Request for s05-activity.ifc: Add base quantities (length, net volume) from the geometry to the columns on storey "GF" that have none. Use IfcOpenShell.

First a look at what the model holds.

```python
import ifcopenshell
import ifcopenshell.util.element
import ifcopenshell.util.unit

model = ifcopenshell.open("s05-activity.ifc")
print(model.schema)
for unit_type in ("LENGTHUNIT", "AREAUNIT", "VOLUMEUNIT"):
    print(unit_type, ifcopenshell.util.unit.calculate_unit_scale(model, unit_type))
storey = next(s for s in model.by_type("IfcBuildingStorey") if s.Name == "GF")
columns = [e for e in ifcopenshell.util.element.get_decomposition(storey) if e.is_a("IfcColumn")]
for e in sorted(columns, key=lambda e: e.id()):
    print(e.id(), e.is_a(), e.Name, list(ifcopenshell.util.element.get_psets(e, qtos_only=True)), sep=" | ")
```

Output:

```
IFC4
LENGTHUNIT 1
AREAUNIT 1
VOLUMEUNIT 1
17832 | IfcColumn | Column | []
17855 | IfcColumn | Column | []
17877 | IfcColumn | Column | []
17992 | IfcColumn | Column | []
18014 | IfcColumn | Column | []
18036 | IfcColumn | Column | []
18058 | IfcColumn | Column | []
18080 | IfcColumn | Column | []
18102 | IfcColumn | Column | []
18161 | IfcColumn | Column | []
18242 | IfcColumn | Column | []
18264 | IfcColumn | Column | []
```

```python
import ifcopenshell
import ifcopenshell.api.pset
import ifcopenshell.geom
import ifcopenshell.util.element
import ifcopenshell.util.shape
import ifcopenshell.util.unit

model = ifcopenshell.open("s05-activity.ifc")
unit_scale = ifcopenshell.util.unit.calculate_unit_scale(model)
volume_scale = ifcopenshell.util.unit.calculate_unit_scale(model, "VOLUMEUNIT")
settings = ifcopenshell.geom.settings()

storey = next(s for s in model.by_type("IfcBuildingStorey") if s.Name == "GF")
columns = [e for e in ifcopenshell.util.element.get_decomposition(storey) if e.is_a("IfcColumn")]

for e in sorted(columns, key=lambda e: e.id()):
    if ifcopenshell.util.element.get_psets(e, qtos_only=True, should_inherit=False):
        continue
    # Geometry comes back in metres, in the element's own axes.
    shape = ifcopenshell.geom.create_shape(settings, e)
    values = {
        "Length": ifcopenshell.util.shape.get_z(shape.geometry) / unit_scale,
        "NetVolume": ifcopenshell.util.shape.get_volume(shape.geometry) / volume_scale,
    }
    qto = ifcopenshell.api.pset.add_qto(model, product=e, name="Qto_ColumnBaseQuantities")
    ifcopenshell.api.pset.edit_qto(model, qto=qto, properties=values)
    print(e.id(), {k: round(v, 3) for k, v in values.items()})

model.write("s05-activity_v2.ifc")
```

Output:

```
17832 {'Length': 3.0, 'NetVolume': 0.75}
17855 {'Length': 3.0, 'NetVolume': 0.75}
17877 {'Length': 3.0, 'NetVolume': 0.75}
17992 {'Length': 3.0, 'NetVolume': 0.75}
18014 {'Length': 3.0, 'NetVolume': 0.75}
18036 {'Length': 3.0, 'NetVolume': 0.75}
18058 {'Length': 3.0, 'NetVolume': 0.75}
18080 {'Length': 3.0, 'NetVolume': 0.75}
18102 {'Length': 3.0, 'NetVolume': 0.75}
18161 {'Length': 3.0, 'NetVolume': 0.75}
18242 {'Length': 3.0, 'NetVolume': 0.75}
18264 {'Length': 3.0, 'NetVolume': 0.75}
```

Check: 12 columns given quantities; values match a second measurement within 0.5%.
